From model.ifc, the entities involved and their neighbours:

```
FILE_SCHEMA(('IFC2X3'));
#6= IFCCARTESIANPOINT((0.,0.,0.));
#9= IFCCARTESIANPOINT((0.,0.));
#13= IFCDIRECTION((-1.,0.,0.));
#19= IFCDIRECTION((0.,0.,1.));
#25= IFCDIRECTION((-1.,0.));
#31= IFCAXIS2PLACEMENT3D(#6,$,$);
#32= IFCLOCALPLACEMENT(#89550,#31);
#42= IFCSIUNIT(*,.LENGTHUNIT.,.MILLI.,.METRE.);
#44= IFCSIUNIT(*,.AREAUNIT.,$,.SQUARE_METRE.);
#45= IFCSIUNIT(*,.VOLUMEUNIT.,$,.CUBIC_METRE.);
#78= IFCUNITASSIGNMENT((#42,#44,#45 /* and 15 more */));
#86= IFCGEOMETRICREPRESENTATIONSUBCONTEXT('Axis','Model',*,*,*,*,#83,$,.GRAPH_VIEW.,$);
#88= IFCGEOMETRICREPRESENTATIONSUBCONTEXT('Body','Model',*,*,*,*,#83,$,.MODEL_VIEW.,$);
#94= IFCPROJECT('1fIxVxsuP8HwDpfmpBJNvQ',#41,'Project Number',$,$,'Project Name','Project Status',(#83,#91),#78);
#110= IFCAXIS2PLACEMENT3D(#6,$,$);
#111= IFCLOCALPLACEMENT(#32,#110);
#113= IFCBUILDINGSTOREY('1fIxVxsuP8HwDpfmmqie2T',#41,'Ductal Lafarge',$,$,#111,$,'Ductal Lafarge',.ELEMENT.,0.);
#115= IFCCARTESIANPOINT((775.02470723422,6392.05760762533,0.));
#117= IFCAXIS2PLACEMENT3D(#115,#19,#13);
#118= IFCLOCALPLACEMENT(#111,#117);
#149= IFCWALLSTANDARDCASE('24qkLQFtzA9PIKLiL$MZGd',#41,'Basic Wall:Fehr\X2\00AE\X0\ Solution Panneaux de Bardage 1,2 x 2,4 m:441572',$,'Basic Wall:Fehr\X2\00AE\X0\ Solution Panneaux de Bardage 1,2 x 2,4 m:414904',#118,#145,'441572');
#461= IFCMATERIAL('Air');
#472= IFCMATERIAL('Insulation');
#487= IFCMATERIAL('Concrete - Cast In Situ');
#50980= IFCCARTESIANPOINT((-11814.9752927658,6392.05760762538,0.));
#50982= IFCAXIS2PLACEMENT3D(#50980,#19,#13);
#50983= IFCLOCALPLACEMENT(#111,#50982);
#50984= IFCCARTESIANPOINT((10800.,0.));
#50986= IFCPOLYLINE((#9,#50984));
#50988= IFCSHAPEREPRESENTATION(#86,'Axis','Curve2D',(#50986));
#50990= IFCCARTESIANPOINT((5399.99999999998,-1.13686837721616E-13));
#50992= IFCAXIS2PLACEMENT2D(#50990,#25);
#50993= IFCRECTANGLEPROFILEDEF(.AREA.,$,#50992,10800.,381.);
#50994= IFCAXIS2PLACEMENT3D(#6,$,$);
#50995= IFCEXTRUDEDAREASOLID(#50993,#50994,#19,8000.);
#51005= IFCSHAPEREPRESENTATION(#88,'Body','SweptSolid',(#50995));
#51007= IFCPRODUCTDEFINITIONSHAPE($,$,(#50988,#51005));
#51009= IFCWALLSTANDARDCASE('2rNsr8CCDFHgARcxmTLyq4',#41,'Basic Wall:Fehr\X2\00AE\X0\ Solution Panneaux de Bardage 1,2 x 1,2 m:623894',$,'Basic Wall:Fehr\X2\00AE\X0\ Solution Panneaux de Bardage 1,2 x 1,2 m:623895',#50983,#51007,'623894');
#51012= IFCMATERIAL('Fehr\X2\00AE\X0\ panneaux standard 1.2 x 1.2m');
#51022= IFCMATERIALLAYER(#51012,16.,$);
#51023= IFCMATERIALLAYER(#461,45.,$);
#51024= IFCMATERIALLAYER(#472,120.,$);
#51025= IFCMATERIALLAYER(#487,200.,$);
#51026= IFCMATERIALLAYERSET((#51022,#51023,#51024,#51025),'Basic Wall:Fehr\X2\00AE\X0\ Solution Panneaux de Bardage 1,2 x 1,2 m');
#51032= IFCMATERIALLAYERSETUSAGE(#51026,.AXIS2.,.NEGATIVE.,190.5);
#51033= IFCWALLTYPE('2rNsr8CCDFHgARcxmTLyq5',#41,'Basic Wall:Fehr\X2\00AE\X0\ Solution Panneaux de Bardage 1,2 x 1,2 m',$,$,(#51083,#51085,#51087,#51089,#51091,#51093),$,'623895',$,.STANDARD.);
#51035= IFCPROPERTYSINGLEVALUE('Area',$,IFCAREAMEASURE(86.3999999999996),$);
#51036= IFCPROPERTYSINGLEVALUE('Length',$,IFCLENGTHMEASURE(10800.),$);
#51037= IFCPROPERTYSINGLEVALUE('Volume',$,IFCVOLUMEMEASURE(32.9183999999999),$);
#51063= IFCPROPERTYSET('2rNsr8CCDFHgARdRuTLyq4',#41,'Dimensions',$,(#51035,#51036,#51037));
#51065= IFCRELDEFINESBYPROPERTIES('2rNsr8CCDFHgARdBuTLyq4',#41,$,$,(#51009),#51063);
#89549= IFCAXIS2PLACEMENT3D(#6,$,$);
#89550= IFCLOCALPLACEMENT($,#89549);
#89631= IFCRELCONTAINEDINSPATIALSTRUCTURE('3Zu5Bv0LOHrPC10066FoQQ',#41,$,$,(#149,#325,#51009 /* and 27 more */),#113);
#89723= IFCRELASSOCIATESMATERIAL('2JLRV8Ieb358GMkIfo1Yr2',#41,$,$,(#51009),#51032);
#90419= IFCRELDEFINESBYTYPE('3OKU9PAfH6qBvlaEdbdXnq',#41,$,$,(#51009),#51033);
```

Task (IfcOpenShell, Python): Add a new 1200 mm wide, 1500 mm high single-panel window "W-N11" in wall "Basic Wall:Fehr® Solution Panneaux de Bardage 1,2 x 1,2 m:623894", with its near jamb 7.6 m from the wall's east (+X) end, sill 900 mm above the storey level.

```python
import numpy as np
import ifcopenshell
import ifcopenshell.api.feature
import ifcopenshell.api.geometry
import ifcopenshell.api.pset
import ifcopenshell.api.root
import ifcopenshell.api.spatial
import ifcopenshell.api.type
import ifcopenshell.geom
import ifcopenshell.util.element
import ifcopenshell.util.placement
import ifcopenshell.util.representation
import ifcopenshell.util.shape
import ifcopenshell.util.unit

model = ifcopenshell.open("model.ifc")
unit_scale = ifcopenshell.util.unit.calculate_unit_scale(model)
area_scale = ifcopenshell.util.unit.calculate_unit_scale(model, "AREAUNIT")
volume_scale = ifcopenshell.util.unit.calculate_unit_scale(model, "VOLUMEUNIT")
settings = ifcopenshell.geom.settings()


def volume(element):
    """Net volume in cubic metres, openings subtracted."""
    shape = ifcopenshell.geom.create_shape(settings, element)
    return ifcopenshell.util.shape.get_volume(shape.geometry)


wall = model.by_id(51009)
storey = ifcopenshell.util.element.get_container(wall, ifc_class="IfcBuildingStorey")
context = ifcopenshell.util.representation.get_context(model, "Model", "Body", "MODEL_VIEW")
before = volume(wall)

width, height, from_end, sill = 1.2, 1.5, 7.6, 0.9  # metres

# The wall runs along its own X axis, and the end named is its -X end.
wall_shape = ifcopenshell.geom.create_shape(settings, wall)
x, y, z = ifcopenshell.util.shape.get_vertices(wall_shape.geometry).T
start = x.min() + from_end
face, thickness = float(y.min()), float(y.max() - y.min())
wall_matrix = ifcopenshell.util.placement.get_local_placement(wall.ObjectPlacement)
level = ifcopenshell.util.placement.get_local_placement(storey.ObjectPlacement)[2, 3]


def in_wall(x, y):
    """Placement at x, y metres in the wall's axes, at sill height."""
    matrix = wall_matrix.copy()
    matrix[:, 3] = wall_matrix @ np.array([x / unit_scale, y / unit_scale, 0.0, 1.0])
    matrix[2, 3] = level + sill / unit_scale
    return matrix


# Opening: a box that overshoots both wall faces by 50 mm.
opening = ifcopenshell.api.root.create_entity(model, ifc_class="IfcOpeningElement")
box = ifcopenshell.api.geometry.add_wall_representation(
    model, context=context, length=width, height=height, thickness=thickness + 0.1
)
ifcopenshell.api.geometry.assign_representation(model, product=opening, representation=box)
ifcopenshell.api.geometry.edit_object_placement(model, product=opening, matrix=in_wall(start, face - 0.05), is_si=False)
ifcopenshell.api.feature.add_feature(model, feature=opening, element=wall)

window = ifcopenshell.api.root.create_entity(model, ifc_class="IfcWindow", name="W-N11")
window.OverallWidth, window.OverallHeight = width / unit_scale, height / unit_scale
body = ifcopenshell.api.geometry.add_window_representation(
    model,
    context=context,
    overall_width=window.OverallWidth,
    overall_height=window.OverallHeight,
    partition_type="SINGLE_PANEL",
)
ifcopenshell.api.geometry.assign_representation(model, product=window, representation=body)
ifcopenshell.api.spatial.assign_container(model, products=[window], relating_structure=storey)
fills = ifcopenshell.api.feature.add_filling(model, opening=opening, element=window)
fills.OwnerHistory = window.OwnerHistory  # required in IFC2X3

# IFC2X3 keeps the operation on the window style.
style = ifcopenshell.api.root.create_entity(model, ifc_class="IfcWindowStyle", name="W-N11")
style.OperationType, style.ConstructionType = "SINGLE_PANEL", "NOTDEFINED"
style.ParameterTakesPrecedence = style.Sizeable = False
ifcopenshell.api.type.assign_type(model, related_objects=[window], relating_type=style)

# Centre the window in the wall's thickness.
ifcopenshell.api.geometry.edit_object_placement(model, product=window, matrix=in_wall(start, face), is_si=False)
window_shape = ifcopenshell.geom.create_shape(settings, window)
depth = ifcopenshell.util.shape.get_vertices(window_shape.geometry)[:, 1]
offset = face + thickness / 2 - (depth.min() + depth.max()) / 2
ifcopenshell.api.geometry.edit_object_placement(model, product=window, matrix=in_wall(start, offset), is_si=False)

after = volume(wall)

# Update the wall's stored quantities.
pset = model.by_id(ifcopenshell.util.element.get_pset(wall, "Dimensions", should_inherit=False)["id"])
ifcopenshell.api.pset.edit_pset(model, pset=pset, properties={
    "Area": model.create_entity("IfcAreaMeasure", after / thickness / area_scale),
    "Volume": model.create_entity("IfcVolumeMeasure", after / volume_scale),
})

print(f"wall volume {before:.3f} -> {after:.3f} m3")

model.write("model_rev.ifc")
```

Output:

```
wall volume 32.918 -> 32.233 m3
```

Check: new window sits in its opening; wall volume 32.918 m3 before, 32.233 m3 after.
